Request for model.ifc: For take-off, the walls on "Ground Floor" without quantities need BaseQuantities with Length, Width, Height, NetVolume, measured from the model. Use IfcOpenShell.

First a look at what the model holds.

```python
import ifcopenshell
import ifcopenshell.util.element
import ifcopenshell.util.unit

model = ifcopenshell.open("model.ifc")
print(model.schema)
for unit_type in ("LENGTHUNIT", "AREAUNIT", "VOLUMEUNIT"):
    print(unit_type, ifcopenshell.util.unit.calculate_unit_scale(model, unit_type))
storey = next(s for s in model.by_type("IfcBuildingStorey") if s.Name == "Ground Floor")
walls = [e for e in ifcopenshell.util.element.get_decomposition(storey) if e.is_a("IfcWall")]
for e in sorted(walls, key=lambda e: e.id()):
    print(e.id(), e.is_a(), e.Name, list(ifcopenshell.util.element.get_psets(e, qtos_only=True)), sep=" | ")
```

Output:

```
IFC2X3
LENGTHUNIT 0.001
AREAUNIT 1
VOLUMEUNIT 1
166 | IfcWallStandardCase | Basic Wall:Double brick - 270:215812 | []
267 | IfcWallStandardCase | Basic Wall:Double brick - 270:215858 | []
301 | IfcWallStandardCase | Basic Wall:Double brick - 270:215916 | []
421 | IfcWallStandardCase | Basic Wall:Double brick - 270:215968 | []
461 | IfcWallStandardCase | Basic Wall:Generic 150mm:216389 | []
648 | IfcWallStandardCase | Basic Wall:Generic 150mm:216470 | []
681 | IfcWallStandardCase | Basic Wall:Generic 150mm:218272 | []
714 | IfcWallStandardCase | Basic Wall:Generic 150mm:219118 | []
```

```python
import ifcopenshell
import ifcopenshell.api.pset
import ifcopenshell.geom
import ifcopenshell.util.element
import ifcopenshell.util.shape
import ifcopenshell.util.unit

model = ifcopenshell.open("model.ifc")
unit_scale = ifcopenshell.util.unit.calculate_unit_scale(model)
volume_scale = ifcopenshell.util.unit.calculate_unit_scale(model, "VOLUMEUNIT")
settings = ifcopenshell.geom.settings()

storey = next(s for s in model.by_type("IfcBuildingStorey") if s.Name == "Ground Floor")
walls = [e for e in ifcopenshell.util.element.get_decomposition(storey) if e.is_a("IfcWall")]

for e in sorted(walls, key=lambda e: e.id()):
    if ifcopenshell.util.element.get_psets(e, qtos_only=True, should_inherit=False):
        continue
    # Geometry comes back in metres, in the element's own axes.
    shape = ifcopenshell.geom.create_shape(settings, e)
    values = {
        "Length": ifcopenshell.util.shape.get_x(shape.geometry) / unit_scale,
        "Width": ifcopenshell.util.shape.get_y(shape.geometry) / unit_scale,
        "Height": ifcopenshell.util.shape.get_z(shape.geometry) / unit_scale,
        "NetVolume": ifcopenshell.util.shape.get_volume(shape.geometry) / volume_scale,
    }
    qto = ifcopenshell.api.pset.add_qto(model, product=e, name="BaseQuantities")
    ifcopenshell.api.pset.edit_qto(model, qto=qto, properties=values)
    print(e.id(), {k: round(v, 3) for k, v in values.items()})

model.write("model_updated.ifc")
```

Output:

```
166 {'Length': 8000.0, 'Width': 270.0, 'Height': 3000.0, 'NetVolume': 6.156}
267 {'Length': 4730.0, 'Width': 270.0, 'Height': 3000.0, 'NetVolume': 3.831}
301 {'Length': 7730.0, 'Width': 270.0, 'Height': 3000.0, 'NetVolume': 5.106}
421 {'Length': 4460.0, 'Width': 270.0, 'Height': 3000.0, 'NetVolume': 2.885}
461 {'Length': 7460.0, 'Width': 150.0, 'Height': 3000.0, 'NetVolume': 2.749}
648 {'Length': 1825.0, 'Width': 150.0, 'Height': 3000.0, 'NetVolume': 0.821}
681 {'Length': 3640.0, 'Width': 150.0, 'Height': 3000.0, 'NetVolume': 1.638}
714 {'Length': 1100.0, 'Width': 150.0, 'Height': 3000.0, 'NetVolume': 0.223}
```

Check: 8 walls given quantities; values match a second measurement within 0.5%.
